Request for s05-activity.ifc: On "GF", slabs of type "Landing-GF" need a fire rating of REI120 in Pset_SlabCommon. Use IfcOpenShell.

First a look at what the model holds.

```python
import ifcopenshell
import ifcopenshell.util.element

model = ifcopenshell.open("s05-activity.ifc")
print(model.schema)
storey = next(s for s in model.by_type("IfcBuildingStorey") if s.Name == "GF")
slabs = [e for e in ifcopenshell.util.element.get_decomposition(storey) if e.is_a("IfcSlab")]
seen = {}
for e in slabs:
    element_type = ifcopenshell.util.element.get_type(e)
    key = (element_type.Name if element_type != e and element_type else None, ifcopenshell.util.element.get_pset(e, "Pset_SlabCommon", "FireRating"))
    seen[key] = seen.get(key, 0) + 1
for (name, value), count in sorted(seen.items(), key=str):
    print(count, "x", name, "|", value)
```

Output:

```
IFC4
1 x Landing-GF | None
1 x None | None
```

```python
import ifcopenshell
import ifcopenshell.api.pset
import ifcopenshell.util.element

model = ifcopenshell.open("s05-activity.ifc")

storey = next(s for s in model.by_type("IfcBuildingStorey") if s.Name == "GF")
slabs = [e for e in ifcopenshell.util.element.get_decomposition(storey) if e.is_a("IfcSlab")]

count = 0
for e in slabs:
    element_type = ifcopenshell.util.element.get_type(e)
    if element_type in (None, e) or element_type.Name != "Landing-GF":
        continue
    # add_pset returns the element's existing set when there is one.
    pset = ifcopenshell.api.pset.add_pset(model, product=e, name="Pset_SlabCommon")
    ifcopenshell.api.pset.edit_pset(model, pset=pset, properties={"FireRating": "REI120"})
    count += 1

print(count, "slabs updated")

model.write("s05-activity_updated.ifc")
```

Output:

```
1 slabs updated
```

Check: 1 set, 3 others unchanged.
